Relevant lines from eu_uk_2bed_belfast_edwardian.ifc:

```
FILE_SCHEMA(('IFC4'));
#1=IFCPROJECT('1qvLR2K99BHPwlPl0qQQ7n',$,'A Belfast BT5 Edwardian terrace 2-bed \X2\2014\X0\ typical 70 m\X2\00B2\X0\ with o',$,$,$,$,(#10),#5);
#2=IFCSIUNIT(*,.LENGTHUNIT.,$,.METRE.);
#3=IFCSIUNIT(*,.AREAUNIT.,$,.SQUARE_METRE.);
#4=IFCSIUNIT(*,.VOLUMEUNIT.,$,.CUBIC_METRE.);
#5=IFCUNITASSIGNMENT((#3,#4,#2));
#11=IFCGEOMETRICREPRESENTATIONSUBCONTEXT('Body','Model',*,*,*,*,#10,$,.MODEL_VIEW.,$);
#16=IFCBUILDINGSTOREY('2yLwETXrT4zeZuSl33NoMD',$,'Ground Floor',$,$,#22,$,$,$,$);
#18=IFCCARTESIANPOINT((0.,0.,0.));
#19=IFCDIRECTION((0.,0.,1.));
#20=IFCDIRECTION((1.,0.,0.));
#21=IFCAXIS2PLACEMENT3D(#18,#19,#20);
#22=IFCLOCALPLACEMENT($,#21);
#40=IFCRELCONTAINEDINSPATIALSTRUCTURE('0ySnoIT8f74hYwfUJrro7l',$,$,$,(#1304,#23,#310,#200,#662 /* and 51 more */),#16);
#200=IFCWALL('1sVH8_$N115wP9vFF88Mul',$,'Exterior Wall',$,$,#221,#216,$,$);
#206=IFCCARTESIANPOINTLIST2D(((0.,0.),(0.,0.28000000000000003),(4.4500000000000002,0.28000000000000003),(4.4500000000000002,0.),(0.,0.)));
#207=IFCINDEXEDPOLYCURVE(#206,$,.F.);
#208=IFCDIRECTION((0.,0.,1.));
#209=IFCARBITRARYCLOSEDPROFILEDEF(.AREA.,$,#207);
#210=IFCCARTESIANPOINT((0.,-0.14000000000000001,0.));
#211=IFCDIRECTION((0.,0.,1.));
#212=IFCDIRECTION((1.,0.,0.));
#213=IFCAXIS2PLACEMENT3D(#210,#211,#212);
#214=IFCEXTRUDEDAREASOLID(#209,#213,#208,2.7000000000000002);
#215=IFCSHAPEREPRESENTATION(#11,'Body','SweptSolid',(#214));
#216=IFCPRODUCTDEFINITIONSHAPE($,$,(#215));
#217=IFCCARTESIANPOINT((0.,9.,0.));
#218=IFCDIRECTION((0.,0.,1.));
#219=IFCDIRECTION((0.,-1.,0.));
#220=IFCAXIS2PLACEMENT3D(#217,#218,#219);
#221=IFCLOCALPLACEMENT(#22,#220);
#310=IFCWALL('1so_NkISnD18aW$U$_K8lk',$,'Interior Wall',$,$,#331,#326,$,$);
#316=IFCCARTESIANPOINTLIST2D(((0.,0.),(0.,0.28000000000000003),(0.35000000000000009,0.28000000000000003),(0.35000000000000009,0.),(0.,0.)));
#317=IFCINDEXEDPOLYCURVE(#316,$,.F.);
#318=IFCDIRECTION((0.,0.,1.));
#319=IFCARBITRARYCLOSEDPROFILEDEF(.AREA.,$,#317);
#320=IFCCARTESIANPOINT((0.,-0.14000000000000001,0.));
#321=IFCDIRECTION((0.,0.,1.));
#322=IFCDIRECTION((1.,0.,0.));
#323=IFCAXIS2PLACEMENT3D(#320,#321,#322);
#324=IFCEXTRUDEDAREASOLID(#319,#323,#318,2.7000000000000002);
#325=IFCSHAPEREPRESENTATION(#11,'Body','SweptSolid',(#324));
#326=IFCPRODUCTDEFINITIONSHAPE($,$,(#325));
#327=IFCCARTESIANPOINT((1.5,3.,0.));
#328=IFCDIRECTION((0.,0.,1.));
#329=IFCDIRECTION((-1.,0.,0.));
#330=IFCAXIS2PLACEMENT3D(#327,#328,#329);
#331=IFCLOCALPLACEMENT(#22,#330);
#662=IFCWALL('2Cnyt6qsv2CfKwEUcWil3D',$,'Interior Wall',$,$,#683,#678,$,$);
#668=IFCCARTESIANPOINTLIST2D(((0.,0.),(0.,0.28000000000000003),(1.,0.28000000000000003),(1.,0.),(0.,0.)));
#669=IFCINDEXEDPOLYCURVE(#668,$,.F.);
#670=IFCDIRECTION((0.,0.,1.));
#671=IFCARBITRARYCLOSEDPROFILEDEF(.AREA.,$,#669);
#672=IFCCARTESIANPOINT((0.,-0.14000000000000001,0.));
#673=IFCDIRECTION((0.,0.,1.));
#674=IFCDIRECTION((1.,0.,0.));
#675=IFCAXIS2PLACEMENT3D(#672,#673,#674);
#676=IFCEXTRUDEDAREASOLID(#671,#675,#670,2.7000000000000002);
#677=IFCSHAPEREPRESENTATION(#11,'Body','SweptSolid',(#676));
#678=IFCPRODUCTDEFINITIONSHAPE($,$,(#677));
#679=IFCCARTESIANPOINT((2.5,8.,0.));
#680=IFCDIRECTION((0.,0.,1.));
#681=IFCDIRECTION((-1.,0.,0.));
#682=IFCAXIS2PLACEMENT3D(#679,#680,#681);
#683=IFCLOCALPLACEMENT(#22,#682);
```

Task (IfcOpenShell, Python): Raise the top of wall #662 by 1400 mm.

```python
import ifcopenshell
import ifcopenshell.geom
import ifcopenshell.util.representation
import ifcopenshell.util.shape

model = ifcopenshell.open("eu_uk_2bed_belfast_edwardian.ifc")
settings = ifcopenshell.geom.settings()


def volume(element):
    """Net volume in cubic metres, openings subtracted."""
    shape = ifcopenshell.geom.create_shape(settings, element)
    return ifcopenshell.util.shape.get_volume(shape.geometry)


wall = model.by_guid("2Cnyt6qsv2CfKwEUcWil3D")
before = volume(wall)

body = ifcopenshell.util.representation.get_representation(wall, "Model", "Body")
solid = body.Items[0]
old_height = solid.Depth
solid.Depth += 1.4
after = volume(wall)

print(f"height {old_height:g} -> {solid.Depth:g}, volume {before:.3f} -> {after:.3f} m3")

model.write("eu_uk_2bed_belfast_edwardian-out.ifc")
```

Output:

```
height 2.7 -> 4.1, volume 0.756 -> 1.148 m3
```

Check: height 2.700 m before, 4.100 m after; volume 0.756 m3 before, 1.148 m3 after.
